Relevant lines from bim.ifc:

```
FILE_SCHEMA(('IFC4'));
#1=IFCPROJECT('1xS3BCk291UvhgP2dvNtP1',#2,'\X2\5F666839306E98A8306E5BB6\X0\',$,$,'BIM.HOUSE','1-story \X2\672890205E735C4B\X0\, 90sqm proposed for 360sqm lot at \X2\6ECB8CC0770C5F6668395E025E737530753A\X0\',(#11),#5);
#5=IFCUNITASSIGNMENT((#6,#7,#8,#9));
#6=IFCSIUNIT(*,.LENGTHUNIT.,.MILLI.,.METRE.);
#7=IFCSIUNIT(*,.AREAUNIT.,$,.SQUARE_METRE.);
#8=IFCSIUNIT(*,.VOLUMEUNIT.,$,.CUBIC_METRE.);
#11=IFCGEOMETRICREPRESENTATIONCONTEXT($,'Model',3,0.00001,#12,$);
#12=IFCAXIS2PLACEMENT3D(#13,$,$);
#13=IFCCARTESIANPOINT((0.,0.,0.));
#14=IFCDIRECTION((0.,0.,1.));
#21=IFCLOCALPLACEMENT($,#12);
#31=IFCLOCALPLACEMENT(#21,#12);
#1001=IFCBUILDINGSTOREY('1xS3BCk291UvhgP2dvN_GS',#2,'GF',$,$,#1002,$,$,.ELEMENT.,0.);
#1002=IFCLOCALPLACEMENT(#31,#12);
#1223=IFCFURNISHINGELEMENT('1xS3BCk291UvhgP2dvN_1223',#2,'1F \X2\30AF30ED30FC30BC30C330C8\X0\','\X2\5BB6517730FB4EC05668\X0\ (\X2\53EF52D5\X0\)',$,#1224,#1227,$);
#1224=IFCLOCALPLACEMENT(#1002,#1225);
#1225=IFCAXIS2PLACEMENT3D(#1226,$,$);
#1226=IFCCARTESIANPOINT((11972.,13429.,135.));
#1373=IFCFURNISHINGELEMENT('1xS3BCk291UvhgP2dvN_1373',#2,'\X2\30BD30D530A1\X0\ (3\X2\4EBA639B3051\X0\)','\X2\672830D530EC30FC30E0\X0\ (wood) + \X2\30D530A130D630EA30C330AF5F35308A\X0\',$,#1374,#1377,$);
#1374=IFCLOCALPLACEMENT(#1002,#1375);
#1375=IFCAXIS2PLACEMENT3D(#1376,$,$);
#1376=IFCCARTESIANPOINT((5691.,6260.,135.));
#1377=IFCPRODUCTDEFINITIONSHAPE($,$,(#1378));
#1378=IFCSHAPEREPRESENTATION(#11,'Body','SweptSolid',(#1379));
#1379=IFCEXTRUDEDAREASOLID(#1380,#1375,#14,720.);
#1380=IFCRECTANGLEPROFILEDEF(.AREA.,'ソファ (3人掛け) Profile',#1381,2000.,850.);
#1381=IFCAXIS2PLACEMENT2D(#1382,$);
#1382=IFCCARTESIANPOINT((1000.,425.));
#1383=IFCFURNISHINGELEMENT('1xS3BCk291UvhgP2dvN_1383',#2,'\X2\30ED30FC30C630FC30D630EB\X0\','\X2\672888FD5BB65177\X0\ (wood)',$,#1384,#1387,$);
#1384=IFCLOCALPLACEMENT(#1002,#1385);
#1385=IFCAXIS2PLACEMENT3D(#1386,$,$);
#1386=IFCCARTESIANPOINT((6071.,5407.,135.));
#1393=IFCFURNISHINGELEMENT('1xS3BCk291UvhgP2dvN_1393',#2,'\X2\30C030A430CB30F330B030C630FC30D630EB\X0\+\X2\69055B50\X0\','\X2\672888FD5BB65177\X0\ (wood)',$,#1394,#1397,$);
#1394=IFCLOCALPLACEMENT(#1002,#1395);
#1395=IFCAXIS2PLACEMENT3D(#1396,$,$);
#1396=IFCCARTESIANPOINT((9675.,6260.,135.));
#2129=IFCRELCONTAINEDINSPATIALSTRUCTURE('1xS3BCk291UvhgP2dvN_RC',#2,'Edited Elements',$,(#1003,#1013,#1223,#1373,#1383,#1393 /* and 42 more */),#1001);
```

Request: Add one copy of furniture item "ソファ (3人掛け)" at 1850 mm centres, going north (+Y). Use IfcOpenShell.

```python
import numpy as np
import ifcopenshell
import ifcopenshell.api.geometry
import ifcopenshell.api.root
import ifcopenshell.util.element
import ifcopenshell.util.placement
import ifcopenshell.util.unit

model = ifcopenshell.open("bim.ifc")
unit_scale = ifcopenshell.util.unit.calculate_unit_scale(model)


def reuse_history(source, copy):
    """copy_class also copies each property set's owner history, people and application; keep the originals."""
    for rel in copy.IsDefinedBy:
        if rel.is_a("IfcRelDefinesByProperties") and (history := rel.RelatingPropertyDefinition.OwnerHistory):
            rel.RelatingPropertyDefinition.OwnerHistory = source.OwnerHistory
            ifcopenshell.util.element.remove_deep2(model, history)


source = model.by_guid("1xS3BCk291UvhgP2dvN_1373")
base = ifcopenshell.util.placement.get_local_placement(source.ObjectPlacement)
step = np.array([0.0, 1.0, 0.0]) * 1.85 / unit_scale

for i in range(1, 2):
    copy = ifcopenshell.api.root.copy_class(model, product=source)
    copy.Representation = ifcopenshell.util.element.copy_deep(
        model, source.Representation, exclude=["IfcGeometricRepresentationContext", "IfcRepresentationMap"]
    )
    reuse_history(source, copy)
    matrix = base.copy()
    matrix[:3, 3] += i * step
    print("added at", matrix[:3, 3].round(3) + 0.0)
    ifcopenshell.api.geometry.edit_object_placement(model, product=copy, matrix=matrix, is_si=False)

model.write("bim_edited.ifc")
```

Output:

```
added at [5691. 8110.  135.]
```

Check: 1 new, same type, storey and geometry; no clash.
